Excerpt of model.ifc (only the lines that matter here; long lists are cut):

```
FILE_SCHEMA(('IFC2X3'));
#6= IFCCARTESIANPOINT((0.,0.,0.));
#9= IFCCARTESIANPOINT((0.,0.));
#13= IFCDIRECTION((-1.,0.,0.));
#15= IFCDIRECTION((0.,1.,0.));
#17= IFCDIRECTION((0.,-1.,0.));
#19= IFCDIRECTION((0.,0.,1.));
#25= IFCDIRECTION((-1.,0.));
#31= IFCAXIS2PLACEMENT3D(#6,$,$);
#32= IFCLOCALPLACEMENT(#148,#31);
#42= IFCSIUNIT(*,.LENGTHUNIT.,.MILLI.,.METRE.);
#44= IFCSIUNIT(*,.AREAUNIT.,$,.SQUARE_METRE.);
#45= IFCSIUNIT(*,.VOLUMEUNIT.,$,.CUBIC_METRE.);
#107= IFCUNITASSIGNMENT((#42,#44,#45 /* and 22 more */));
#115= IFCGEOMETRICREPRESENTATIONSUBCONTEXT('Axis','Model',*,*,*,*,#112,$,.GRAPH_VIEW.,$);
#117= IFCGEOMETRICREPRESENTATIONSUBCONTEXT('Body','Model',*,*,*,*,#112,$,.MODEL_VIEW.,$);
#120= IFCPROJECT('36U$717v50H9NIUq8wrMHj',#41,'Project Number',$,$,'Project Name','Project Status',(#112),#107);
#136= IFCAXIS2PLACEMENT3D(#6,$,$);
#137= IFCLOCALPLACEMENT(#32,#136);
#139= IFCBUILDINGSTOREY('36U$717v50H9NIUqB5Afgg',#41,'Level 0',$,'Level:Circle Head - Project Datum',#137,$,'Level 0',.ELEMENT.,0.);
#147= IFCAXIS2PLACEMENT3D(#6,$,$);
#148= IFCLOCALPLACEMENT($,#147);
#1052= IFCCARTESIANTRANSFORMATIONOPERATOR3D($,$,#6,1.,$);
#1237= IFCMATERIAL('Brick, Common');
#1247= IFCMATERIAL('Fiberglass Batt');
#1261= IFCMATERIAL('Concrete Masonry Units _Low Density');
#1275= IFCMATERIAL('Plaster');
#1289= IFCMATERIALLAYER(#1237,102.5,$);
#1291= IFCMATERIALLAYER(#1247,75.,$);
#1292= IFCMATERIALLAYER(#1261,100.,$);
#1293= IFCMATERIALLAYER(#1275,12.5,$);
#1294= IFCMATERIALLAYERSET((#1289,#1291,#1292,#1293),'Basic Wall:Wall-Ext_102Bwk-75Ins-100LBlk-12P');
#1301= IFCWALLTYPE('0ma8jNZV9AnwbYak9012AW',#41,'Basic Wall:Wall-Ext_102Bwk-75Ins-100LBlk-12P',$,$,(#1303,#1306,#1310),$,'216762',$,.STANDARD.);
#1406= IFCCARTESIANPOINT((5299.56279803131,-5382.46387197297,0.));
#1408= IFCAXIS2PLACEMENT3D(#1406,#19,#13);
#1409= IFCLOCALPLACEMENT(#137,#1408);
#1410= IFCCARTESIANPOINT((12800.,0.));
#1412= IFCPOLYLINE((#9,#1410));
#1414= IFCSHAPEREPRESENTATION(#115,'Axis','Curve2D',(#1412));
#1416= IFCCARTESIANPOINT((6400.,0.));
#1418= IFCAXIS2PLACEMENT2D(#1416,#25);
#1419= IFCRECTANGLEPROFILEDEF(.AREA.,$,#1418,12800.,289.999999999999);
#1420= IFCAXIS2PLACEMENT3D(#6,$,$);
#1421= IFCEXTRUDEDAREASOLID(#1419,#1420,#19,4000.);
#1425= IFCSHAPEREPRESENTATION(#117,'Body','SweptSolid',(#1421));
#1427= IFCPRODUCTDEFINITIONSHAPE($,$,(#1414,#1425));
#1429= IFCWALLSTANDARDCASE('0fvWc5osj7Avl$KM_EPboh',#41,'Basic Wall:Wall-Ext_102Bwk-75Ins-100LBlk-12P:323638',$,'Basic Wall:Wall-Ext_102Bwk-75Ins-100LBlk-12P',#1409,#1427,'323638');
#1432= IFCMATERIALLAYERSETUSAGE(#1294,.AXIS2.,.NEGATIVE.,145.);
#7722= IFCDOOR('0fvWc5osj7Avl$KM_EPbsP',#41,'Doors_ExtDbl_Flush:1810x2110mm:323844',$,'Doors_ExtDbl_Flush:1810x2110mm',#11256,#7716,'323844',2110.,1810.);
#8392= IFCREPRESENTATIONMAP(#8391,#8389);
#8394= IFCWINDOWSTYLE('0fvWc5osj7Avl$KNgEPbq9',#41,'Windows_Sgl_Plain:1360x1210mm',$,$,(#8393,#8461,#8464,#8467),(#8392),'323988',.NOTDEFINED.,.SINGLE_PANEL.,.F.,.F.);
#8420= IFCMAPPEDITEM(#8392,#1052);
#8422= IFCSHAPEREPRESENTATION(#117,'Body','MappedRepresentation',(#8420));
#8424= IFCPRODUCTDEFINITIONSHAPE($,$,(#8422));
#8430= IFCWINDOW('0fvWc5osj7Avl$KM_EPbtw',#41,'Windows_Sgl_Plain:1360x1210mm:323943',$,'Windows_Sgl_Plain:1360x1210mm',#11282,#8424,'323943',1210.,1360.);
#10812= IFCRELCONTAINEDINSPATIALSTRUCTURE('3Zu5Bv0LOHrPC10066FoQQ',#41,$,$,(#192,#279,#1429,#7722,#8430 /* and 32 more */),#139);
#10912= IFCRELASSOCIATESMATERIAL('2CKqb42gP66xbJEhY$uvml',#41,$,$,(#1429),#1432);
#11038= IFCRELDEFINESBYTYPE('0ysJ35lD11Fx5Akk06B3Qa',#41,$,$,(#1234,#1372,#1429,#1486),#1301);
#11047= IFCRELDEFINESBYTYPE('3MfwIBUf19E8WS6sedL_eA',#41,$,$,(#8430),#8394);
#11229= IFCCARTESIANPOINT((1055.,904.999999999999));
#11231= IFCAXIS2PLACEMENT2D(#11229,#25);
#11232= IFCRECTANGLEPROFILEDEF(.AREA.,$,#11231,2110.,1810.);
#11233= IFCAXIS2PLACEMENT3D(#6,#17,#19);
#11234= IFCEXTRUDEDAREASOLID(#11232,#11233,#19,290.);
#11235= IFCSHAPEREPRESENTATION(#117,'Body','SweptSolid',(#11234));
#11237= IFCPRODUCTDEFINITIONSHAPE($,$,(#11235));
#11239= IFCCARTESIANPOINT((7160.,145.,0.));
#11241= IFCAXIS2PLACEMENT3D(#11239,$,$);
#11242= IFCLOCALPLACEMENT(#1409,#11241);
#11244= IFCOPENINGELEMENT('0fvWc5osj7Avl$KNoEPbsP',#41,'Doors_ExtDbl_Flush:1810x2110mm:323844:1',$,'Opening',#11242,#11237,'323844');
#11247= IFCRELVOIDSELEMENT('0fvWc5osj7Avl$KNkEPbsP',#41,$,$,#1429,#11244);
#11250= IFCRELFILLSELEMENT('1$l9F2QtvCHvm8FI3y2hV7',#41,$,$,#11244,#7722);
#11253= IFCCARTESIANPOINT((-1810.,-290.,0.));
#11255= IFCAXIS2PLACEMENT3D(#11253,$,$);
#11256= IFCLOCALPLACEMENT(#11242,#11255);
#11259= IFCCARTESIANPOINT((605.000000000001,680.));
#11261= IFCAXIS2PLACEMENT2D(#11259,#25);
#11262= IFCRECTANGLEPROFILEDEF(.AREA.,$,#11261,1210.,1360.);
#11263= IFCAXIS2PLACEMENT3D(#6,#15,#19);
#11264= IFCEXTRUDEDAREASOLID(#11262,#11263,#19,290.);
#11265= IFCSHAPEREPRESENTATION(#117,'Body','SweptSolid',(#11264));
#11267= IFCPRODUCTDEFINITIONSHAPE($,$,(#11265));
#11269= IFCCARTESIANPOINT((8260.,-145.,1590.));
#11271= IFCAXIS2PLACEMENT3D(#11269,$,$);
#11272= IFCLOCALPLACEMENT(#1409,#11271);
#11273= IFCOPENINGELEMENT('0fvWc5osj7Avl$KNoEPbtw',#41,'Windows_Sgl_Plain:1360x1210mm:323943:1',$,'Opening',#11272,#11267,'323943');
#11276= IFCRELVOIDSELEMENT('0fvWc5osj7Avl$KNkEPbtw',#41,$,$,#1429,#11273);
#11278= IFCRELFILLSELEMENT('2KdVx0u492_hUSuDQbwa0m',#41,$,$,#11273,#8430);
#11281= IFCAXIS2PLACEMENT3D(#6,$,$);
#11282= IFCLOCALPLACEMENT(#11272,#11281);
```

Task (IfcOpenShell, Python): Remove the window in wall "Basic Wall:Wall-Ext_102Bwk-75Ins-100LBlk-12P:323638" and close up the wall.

```python
import ifcopenshell
import ifcopenshell.api.feature
import ifcopenshell.api.root
import ifcopenshell.geom
import ifcopenshell.util.shape

model = ifcopenshell.open("model.ifc")
settings = ifcopenshell.geom.settings()


def volume(element):
    """Net volume in cubic metres, openings subtracted."""
    shape = ifcopenshell.geom.create_shape(settings, element)
    return ifcopenshell.util.shape.get_volume(shape.geometry)


window = model.by_guid("0fvWc5osj7Avl$KM_EPbtw")
opening = window.FillsVoids[0].RelatingOpeningElement
wall = opening.VoidsElements[0].RelatingBuildingElement
before = volume(wall)

ifcopenshell.api.root.remove_product(model, product=window)
ifcopenshell.api.feature.remove_feature(model, feature=opening)

after = volume(wall)

print(f"wall volume {before:.3f} -> {after:.3f} m3")

model.write("model_v2.ifc")
```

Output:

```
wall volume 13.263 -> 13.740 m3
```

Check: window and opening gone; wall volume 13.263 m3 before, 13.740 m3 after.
